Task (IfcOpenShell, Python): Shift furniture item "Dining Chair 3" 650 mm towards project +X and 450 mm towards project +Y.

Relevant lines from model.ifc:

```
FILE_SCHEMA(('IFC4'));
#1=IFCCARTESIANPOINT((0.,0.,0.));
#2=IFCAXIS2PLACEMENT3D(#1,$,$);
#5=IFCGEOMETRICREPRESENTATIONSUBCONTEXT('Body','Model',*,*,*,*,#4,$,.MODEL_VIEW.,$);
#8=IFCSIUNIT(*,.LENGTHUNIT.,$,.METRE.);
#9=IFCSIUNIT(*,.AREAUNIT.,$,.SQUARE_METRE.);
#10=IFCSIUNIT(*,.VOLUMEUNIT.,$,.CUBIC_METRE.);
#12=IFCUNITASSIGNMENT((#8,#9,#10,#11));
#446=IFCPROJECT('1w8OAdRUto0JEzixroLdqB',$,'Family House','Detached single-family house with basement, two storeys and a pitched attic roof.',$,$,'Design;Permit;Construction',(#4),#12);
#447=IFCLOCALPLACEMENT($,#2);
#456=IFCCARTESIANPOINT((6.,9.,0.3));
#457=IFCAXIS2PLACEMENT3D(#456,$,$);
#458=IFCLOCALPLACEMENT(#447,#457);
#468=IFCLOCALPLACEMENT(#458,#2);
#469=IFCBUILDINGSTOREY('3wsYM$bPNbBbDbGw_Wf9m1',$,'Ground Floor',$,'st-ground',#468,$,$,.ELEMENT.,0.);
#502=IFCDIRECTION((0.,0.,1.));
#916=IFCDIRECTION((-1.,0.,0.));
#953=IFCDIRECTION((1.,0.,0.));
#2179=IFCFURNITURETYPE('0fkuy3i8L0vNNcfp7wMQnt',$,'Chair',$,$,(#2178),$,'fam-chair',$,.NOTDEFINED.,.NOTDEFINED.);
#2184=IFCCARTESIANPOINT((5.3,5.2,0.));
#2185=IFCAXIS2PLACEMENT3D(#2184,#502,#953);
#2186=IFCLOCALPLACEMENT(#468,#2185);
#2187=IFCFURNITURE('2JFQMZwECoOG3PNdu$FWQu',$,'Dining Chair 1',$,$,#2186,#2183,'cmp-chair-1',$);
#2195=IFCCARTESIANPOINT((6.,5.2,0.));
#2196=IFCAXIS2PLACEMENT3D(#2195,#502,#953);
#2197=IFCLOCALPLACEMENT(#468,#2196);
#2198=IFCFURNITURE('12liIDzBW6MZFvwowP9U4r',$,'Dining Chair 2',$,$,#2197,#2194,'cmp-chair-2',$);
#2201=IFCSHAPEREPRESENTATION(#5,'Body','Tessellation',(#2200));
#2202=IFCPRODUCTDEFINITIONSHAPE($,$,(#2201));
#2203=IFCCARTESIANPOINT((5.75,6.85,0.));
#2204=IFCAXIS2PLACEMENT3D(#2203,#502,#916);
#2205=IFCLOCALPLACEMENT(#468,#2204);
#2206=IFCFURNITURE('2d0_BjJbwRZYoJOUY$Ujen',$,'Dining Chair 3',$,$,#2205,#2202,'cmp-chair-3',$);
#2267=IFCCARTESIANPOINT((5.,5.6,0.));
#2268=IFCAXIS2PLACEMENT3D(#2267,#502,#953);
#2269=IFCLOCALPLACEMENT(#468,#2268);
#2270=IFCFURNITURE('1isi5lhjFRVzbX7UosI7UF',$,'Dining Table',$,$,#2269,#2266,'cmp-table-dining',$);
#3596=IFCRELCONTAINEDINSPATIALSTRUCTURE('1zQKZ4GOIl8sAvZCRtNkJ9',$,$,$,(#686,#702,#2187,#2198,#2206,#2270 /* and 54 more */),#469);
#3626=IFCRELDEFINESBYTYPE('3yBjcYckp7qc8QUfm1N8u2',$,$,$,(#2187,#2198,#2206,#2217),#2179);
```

```python
import ifcopenshell
import ifcopenshell.api.geometry
import ifcopenshell.util.placement

model = ifcopenshell.open("model.ifc")

item = model.by_guid("2d0_BjJbwRZYoJOUY$Ujen")
matrix = ifcopenshell.util.placement.get_local_placement(item.ObjectPlacement)
matrix[0, 3] += 0.65
matrix[1, 3] += 0.45
ifcopenshell.api.geometry.edit_object_placement(model, product=item, matrix=matrix, is_si=False)

print(ifcopenshell.util.placement.get_local_placement(item.ObjectPlacement).round(3) + 0.0)

model.write("model_v2.ifc")
```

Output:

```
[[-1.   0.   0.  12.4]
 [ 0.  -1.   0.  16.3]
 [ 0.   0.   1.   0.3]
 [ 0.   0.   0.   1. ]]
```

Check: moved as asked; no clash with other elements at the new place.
